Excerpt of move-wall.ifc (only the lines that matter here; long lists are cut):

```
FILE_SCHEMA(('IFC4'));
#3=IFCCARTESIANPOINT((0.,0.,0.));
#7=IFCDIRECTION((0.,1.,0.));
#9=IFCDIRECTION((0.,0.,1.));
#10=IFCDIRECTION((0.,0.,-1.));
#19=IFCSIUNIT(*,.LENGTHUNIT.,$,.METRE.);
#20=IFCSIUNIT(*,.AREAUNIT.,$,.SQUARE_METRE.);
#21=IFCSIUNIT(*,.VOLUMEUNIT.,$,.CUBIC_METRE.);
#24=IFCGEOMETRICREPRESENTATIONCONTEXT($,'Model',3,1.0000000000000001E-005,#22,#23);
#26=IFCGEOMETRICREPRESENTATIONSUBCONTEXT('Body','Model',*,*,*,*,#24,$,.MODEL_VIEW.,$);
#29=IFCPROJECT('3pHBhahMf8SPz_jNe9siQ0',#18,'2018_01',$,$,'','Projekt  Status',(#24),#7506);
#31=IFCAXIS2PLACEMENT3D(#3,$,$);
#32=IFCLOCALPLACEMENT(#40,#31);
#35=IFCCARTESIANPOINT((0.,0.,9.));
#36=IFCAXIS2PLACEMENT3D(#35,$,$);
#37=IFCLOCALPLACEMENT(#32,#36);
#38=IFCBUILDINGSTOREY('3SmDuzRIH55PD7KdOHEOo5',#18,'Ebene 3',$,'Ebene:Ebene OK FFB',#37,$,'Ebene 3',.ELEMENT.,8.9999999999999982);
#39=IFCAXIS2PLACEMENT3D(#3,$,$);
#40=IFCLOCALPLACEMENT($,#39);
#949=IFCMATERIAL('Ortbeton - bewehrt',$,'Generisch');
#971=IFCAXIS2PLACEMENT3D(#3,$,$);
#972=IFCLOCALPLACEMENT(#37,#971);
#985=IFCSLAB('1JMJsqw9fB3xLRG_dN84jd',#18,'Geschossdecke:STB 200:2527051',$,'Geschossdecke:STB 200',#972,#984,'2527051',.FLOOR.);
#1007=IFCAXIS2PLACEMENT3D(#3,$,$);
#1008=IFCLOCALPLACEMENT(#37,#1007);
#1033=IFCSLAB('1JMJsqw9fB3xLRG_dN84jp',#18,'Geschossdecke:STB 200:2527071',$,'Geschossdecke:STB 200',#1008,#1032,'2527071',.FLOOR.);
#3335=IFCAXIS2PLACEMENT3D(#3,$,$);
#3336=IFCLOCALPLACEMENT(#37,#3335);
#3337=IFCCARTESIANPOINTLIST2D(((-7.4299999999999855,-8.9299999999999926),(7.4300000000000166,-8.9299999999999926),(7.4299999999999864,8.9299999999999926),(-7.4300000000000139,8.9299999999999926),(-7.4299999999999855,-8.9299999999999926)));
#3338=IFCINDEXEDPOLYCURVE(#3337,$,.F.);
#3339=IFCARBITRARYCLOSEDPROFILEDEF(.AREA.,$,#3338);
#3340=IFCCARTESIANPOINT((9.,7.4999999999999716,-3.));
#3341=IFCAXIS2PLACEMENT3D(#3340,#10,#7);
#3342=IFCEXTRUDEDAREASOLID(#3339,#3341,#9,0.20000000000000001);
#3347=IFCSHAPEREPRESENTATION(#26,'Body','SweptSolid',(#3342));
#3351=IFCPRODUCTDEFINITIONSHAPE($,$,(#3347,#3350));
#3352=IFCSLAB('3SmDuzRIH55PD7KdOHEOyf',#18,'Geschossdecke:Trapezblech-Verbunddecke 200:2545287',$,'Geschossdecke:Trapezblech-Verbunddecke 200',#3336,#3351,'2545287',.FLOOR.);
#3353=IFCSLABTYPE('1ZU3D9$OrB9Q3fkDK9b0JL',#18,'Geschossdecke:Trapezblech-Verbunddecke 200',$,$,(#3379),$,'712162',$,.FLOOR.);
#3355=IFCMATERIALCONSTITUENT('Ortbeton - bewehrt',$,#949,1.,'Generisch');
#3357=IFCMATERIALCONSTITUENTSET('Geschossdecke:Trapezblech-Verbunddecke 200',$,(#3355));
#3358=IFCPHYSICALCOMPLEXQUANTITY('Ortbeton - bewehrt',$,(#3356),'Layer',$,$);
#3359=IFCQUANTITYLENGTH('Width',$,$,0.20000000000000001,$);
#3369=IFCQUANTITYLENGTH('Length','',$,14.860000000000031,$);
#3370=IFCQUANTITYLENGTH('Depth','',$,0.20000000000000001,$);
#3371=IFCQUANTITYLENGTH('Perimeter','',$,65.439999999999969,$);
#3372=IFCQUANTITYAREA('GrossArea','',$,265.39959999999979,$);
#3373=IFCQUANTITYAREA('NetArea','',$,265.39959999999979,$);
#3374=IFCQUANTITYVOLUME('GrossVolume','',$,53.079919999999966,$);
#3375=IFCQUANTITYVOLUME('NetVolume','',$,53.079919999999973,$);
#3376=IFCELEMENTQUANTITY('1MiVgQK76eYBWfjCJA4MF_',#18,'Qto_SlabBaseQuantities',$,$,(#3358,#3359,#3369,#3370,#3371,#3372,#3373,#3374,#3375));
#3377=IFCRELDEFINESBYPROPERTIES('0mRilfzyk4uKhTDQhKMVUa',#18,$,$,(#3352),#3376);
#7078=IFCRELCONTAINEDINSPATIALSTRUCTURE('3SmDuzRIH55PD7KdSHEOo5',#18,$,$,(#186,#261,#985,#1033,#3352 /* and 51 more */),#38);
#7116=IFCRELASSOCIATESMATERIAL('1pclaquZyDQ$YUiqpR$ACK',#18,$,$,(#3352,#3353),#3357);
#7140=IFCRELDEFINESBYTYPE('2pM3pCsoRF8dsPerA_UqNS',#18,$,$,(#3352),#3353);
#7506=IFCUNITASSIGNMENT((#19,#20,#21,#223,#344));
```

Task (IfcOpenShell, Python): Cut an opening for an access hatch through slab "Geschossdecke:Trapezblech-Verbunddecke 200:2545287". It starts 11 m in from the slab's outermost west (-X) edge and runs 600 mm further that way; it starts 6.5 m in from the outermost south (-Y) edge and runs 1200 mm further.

```python
import numpy as np
import ifcopenshell
import ifcopenshell.api.feature
import ifcopenshell.api.geometry
import ifcopenshell.api.pset
import ifcopenshell.api.root
import ifcopenshell.geom
import ifcopenshell.util.element
import ifcopenshell.util.placement
import ifcopenshell.util.representation
import ifcopenshell.util.shape
import ifcopenshell.util.unit

model = ifcopenshell.open("move-wall.ifc")
unit_scale = ifcopenshell.util.unit.calculate_unit_scale(model)
area_scale = ifcopenshell.util.unit.calculate_unit_scale(model, "AREAUNIT")
volume_scale = ifcopenshell.util.unit.calculate_unit_scale(model, "VOLUMEUNIT")
settings = ifcopenshell.geom.settings()


def volume(element):
    """Net volume in cubic metres, openings subtracted."""
    shape = ifcopenshell.geom.create_shape(settings, element)
    return ifcopenshell.util.shape.get_volume(shape.geometry)


slab = model.by_guid("3SmDuzRIH55PD7KdOHEOyf")
before = volume(slab)

# Extent in the slab's own axes, in metres. The edges named are its -X and -Y sides.
slab_shape = ifcopenshell.geom.create_shape(settings, slab)
vertices = ifcopenshell.util.shape.get_vertices(slab_shape.geometry)
x_min, y_min, bottom = vertices.min(axis=0)
top = vertices[:, 2].max()

opening = ifcopenshell.api.root.create_entity(model, ifc_class="IfcOpeningElement", name="Access hatch opening", predefined_type="OPENING")
context = ifcopenshell.util.representation.get_context(model, "Model", "Body", "MODEL_VIEW")
width, depth = 0.6, 1.2
outline = [(0.0, 0.0), (width, 0.0), (width, depth), (0.0, depth), (0.0, 0.0)]
# Overshoot both faces by 50 mm so the cut is clean.
shape = ifcopenshell.api.geometry.add_slab_representation(
    model, context=context, depth=top - bottom + 0.1, polyline=outline
)
ifcopenshell.api.geometry.assign_representation(model, product=opening, representation=shape)

matrix = ifcopenshell.util.placement.get_local_placement(slab.ObjectPlacement)
matrix[:, 3] = matrix @ np.append(np.array([x_min + 11, y_min + 6.5, bottom - 0.05]) / unit_scale, 1.0)
ifcopenshell.api.geometry.edit_object_placement(model, product=opening, matrix=matrix, is_si=False)
ifcopenshell.api.feature.add_feature(model, feature=opening, element=slab)

after = volume(slab)

# Update the slab's stored quantities.
qto = model.by_id(ifcopenshell.util.element.get_pset(slab, "Qto_SlabBaseQuantities", should_inherit=False)["id"])
ifcopenshell.api.pset.edit_qto(model, qto=qto, properties={
    "NetArea": after / (top - bottom) / area_scale,
    "NetVolume": after / volume_scale,
})

print(f"slab volume {before:.3f} -> {after:.3f} m3")

model.write("move-wall_updated.ifc")
```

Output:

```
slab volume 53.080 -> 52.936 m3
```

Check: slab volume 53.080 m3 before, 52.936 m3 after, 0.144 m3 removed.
